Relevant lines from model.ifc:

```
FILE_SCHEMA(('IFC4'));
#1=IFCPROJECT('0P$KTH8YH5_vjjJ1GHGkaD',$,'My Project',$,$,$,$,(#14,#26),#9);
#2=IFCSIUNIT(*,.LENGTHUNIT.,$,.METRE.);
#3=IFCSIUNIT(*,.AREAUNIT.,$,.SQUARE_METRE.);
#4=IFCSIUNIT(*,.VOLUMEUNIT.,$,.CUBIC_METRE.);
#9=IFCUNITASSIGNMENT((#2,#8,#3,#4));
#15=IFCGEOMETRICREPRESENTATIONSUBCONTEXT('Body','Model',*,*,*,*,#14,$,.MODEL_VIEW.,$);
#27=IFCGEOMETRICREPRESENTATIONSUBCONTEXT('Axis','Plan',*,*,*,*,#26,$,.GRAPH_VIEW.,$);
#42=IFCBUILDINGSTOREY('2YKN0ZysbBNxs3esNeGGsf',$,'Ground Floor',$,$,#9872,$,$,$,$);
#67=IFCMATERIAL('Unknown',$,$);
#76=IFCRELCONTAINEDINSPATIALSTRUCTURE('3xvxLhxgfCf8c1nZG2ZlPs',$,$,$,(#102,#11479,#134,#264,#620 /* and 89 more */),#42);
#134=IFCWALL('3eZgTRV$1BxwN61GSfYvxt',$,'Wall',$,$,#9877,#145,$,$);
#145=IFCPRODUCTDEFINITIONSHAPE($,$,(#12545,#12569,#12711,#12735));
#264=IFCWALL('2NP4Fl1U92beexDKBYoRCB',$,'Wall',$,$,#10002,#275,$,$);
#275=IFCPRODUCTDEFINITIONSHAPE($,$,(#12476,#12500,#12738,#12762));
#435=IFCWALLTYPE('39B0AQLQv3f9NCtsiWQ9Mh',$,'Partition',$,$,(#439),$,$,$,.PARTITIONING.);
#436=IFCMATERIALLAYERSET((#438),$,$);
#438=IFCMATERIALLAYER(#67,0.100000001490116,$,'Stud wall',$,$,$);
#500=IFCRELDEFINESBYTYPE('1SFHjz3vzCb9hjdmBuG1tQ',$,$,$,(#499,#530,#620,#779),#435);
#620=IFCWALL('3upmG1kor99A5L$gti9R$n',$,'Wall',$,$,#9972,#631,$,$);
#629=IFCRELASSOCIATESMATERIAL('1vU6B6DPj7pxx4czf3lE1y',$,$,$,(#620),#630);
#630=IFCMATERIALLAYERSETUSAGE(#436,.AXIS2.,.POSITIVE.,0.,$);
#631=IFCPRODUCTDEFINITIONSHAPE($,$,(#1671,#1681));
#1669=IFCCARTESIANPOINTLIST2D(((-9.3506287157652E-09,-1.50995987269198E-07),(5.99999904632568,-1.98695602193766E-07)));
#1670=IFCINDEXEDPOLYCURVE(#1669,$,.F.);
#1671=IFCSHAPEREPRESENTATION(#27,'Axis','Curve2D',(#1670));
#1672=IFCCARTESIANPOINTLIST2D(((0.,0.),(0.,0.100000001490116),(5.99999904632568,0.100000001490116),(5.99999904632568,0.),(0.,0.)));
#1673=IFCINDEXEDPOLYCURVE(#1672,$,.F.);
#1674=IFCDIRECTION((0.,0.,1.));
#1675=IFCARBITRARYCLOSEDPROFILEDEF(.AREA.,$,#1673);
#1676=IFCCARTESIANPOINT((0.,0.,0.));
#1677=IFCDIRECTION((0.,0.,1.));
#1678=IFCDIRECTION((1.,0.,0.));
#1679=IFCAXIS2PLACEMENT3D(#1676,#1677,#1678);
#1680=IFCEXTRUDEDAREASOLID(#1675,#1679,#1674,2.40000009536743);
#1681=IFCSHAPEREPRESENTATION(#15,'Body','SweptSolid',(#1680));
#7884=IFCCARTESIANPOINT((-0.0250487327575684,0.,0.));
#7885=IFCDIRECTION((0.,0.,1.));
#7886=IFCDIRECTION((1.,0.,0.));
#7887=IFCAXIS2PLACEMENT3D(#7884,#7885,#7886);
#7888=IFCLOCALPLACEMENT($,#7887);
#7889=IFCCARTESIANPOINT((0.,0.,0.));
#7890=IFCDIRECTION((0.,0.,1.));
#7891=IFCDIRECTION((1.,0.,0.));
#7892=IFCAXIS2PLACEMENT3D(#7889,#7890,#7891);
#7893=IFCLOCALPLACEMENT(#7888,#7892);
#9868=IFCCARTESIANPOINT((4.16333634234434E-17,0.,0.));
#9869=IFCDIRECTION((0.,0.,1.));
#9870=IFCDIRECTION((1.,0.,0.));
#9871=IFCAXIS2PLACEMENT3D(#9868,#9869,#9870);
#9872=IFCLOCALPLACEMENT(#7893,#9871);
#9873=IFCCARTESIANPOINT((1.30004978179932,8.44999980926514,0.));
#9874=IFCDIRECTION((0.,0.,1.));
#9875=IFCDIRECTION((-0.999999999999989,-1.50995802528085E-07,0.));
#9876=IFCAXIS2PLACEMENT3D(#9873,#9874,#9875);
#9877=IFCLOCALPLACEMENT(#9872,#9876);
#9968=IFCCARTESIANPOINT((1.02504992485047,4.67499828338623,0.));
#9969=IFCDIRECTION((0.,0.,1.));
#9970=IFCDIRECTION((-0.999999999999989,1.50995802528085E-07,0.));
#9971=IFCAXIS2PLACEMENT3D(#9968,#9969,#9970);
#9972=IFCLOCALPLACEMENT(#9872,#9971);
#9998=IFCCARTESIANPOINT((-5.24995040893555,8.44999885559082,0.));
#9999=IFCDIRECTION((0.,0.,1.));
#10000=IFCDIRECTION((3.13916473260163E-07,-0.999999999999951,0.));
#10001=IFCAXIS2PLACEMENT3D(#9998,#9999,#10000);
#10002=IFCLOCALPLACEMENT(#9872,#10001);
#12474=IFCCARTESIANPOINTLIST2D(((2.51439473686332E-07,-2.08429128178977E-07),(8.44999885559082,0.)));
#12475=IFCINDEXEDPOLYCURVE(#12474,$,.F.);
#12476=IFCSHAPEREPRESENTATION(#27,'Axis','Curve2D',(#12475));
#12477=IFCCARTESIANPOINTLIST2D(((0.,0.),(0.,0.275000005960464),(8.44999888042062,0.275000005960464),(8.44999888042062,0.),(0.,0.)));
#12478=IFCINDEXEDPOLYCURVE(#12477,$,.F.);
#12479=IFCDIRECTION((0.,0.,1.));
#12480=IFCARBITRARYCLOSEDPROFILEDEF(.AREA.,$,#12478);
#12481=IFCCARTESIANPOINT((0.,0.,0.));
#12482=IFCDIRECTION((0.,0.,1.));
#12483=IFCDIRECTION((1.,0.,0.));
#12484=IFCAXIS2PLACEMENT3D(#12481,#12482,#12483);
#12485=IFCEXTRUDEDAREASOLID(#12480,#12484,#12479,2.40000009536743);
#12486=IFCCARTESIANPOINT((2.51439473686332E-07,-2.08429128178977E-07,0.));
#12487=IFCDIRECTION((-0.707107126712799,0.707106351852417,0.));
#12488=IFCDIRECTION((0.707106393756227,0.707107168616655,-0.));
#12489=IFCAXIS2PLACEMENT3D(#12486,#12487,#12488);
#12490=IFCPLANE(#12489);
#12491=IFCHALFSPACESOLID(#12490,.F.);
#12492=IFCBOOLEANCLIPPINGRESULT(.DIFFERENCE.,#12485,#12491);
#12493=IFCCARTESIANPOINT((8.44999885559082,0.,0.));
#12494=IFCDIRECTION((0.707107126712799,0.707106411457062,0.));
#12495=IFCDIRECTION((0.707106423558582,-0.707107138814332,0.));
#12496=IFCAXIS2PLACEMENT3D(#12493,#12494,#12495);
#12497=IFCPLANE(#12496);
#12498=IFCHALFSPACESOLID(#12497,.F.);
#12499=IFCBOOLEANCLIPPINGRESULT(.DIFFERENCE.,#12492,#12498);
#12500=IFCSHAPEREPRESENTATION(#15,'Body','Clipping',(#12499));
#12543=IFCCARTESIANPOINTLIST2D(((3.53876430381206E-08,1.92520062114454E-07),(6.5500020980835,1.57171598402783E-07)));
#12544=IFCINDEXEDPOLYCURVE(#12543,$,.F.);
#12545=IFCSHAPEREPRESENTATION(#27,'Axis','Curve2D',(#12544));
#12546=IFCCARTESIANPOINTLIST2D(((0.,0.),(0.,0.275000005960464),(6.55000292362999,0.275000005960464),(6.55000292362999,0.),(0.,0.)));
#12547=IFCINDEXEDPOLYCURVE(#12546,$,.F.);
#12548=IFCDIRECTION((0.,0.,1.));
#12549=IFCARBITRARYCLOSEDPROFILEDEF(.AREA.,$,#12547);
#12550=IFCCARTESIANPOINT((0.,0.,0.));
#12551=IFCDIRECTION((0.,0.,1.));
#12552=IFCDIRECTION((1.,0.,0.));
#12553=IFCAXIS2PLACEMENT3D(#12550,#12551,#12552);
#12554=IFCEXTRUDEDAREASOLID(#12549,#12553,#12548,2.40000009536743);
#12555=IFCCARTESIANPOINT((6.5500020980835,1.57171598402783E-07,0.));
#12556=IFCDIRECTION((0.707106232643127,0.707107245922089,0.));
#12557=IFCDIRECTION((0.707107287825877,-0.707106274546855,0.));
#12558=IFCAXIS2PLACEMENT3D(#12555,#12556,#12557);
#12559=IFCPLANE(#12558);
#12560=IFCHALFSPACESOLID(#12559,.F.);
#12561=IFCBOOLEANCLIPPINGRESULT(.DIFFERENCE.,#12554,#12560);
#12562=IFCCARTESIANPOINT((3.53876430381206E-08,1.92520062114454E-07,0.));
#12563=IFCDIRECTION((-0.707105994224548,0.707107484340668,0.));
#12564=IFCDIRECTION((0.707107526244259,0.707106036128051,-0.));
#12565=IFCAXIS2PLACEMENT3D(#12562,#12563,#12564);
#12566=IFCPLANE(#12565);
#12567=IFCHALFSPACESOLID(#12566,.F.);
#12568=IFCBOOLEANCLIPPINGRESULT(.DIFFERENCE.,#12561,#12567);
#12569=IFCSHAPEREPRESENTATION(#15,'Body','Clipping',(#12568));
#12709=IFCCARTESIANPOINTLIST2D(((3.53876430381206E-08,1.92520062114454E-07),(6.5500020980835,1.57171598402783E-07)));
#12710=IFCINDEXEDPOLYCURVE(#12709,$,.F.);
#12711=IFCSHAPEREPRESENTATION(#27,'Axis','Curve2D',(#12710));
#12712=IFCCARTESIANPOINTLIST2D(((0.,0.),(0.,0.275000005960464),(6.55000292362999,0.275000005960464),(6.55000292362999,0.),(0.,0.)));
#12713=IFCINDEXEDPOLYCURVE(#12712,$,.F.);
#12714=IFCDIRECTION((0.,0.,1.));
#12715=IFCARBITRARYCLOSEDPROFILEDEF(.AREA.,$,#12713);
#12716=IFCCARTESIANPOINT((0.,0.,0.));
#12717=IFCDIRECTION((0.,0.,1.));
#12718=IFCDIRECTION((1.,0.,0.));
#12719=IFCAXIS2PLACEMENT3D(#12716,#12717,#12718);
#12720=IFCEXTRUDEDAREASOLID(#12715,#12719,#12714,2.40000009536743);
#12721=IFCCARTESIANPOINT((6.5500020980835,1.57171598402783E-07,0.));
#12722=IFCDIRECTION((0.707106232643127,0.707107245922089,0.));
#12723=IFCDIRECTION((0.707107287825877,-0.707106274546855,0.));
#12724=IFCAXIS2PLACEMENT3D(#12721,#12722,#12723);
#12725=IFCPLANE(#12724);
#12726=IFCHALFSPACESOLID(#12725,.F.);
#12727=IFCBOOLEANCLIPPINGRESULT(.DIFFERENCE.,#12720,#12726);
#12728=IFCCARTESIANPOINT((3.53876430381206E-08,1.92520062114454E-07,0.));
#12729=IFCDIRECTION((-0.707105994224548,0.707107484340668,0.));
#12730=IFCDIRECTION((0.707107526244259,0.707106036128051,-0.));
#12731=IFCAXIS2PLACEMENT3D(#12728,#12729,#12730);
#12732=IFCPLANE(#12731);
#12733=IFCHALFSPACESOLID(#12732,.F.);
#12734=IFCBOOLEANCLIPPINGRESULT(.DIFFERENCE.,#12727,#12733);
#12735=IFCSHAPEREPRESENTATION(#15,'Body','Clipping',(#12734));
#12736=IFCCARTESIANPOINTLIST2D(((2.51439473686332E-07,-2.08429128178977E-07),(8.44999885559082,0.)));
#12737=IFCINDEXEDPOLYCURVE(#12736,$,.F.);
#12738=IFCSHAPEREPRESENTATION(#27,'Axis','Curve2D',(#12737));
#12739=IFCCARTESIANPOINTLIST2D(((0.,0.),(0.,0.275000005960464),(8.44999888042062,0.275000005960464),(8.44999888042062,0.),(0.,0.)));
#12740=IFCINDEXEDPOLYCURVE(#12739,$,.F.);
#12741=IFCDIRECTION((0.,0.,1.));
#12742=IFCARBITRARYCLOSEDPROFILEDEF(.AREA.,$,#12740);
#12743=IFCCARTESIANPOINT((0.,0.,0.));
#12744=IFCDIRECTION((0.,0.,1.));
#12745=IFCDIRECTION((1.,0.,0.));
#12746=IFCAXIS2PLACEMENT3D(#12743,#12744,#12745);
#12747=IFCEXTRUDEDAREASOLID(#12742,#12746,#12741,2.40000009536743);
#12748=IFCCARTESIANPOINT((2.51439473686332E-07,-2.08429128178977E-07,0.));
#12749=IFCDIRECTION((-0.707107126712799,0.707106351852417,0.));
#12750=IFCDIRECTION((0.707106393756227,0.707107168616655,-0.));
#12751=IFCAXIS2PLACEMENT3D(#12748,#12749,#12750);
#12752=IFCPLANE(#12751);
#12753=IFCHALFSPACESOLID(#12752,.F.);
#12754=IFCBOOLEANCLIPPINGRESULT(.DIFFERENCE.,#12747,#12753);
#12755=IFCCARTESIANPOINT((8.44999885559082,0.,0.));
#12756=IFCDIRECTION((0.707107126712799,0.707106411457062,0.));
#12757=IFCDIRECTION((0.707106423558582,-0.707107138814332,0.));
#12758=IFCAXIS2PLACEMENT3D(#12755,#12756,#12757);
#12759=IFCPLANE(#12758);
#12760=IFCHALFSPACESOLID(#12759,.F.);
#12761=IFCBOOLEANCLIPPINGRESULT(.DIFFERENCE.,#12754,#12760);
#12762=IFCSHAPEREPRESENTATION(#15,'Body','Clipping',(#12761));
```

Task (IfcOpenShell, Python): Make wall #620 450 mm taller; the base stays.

```python
import ifcopenshell
import ifcopenshell.geom
import ifcopenshell.util.representation
import ifcopenshell.util.shape
import ifcopenshell.util.unit

model = ifcopenshell.open("model.ifc")
unit_scale = ifcopenshell.util.unit.calculate_unit_scale(model)
settings = ifcopenshell.geom.settings()


def volume(element):
    """Net volume in cubic metres, openings subtracted."""
    shape = ifcopenshell.geom.create_shape(settings, element)
    return ifcopenshell.util.shape.get_volume(shape.geometry)


wall = model.by_guid("3upmG1kor99A5L$gti9R$n")
before = volume(wall)

body = ifcopenshell.util.representation.get_representation(wall, "Model", "Body")
solid = body.Items[0]
old_height = solid.Depth
solid.Depth += 0.45 / unit_scale
after = volume(wall)

print(f"height {old_height:g} -> {solid.Depth:g}, volume {before:.3f} -> {after:.3f} m3")

model.write("model_updated.ifc")
```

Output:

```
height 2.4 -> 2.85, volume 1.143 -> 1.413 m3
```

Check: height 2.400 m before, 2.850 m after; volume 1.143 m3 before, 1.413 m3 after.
